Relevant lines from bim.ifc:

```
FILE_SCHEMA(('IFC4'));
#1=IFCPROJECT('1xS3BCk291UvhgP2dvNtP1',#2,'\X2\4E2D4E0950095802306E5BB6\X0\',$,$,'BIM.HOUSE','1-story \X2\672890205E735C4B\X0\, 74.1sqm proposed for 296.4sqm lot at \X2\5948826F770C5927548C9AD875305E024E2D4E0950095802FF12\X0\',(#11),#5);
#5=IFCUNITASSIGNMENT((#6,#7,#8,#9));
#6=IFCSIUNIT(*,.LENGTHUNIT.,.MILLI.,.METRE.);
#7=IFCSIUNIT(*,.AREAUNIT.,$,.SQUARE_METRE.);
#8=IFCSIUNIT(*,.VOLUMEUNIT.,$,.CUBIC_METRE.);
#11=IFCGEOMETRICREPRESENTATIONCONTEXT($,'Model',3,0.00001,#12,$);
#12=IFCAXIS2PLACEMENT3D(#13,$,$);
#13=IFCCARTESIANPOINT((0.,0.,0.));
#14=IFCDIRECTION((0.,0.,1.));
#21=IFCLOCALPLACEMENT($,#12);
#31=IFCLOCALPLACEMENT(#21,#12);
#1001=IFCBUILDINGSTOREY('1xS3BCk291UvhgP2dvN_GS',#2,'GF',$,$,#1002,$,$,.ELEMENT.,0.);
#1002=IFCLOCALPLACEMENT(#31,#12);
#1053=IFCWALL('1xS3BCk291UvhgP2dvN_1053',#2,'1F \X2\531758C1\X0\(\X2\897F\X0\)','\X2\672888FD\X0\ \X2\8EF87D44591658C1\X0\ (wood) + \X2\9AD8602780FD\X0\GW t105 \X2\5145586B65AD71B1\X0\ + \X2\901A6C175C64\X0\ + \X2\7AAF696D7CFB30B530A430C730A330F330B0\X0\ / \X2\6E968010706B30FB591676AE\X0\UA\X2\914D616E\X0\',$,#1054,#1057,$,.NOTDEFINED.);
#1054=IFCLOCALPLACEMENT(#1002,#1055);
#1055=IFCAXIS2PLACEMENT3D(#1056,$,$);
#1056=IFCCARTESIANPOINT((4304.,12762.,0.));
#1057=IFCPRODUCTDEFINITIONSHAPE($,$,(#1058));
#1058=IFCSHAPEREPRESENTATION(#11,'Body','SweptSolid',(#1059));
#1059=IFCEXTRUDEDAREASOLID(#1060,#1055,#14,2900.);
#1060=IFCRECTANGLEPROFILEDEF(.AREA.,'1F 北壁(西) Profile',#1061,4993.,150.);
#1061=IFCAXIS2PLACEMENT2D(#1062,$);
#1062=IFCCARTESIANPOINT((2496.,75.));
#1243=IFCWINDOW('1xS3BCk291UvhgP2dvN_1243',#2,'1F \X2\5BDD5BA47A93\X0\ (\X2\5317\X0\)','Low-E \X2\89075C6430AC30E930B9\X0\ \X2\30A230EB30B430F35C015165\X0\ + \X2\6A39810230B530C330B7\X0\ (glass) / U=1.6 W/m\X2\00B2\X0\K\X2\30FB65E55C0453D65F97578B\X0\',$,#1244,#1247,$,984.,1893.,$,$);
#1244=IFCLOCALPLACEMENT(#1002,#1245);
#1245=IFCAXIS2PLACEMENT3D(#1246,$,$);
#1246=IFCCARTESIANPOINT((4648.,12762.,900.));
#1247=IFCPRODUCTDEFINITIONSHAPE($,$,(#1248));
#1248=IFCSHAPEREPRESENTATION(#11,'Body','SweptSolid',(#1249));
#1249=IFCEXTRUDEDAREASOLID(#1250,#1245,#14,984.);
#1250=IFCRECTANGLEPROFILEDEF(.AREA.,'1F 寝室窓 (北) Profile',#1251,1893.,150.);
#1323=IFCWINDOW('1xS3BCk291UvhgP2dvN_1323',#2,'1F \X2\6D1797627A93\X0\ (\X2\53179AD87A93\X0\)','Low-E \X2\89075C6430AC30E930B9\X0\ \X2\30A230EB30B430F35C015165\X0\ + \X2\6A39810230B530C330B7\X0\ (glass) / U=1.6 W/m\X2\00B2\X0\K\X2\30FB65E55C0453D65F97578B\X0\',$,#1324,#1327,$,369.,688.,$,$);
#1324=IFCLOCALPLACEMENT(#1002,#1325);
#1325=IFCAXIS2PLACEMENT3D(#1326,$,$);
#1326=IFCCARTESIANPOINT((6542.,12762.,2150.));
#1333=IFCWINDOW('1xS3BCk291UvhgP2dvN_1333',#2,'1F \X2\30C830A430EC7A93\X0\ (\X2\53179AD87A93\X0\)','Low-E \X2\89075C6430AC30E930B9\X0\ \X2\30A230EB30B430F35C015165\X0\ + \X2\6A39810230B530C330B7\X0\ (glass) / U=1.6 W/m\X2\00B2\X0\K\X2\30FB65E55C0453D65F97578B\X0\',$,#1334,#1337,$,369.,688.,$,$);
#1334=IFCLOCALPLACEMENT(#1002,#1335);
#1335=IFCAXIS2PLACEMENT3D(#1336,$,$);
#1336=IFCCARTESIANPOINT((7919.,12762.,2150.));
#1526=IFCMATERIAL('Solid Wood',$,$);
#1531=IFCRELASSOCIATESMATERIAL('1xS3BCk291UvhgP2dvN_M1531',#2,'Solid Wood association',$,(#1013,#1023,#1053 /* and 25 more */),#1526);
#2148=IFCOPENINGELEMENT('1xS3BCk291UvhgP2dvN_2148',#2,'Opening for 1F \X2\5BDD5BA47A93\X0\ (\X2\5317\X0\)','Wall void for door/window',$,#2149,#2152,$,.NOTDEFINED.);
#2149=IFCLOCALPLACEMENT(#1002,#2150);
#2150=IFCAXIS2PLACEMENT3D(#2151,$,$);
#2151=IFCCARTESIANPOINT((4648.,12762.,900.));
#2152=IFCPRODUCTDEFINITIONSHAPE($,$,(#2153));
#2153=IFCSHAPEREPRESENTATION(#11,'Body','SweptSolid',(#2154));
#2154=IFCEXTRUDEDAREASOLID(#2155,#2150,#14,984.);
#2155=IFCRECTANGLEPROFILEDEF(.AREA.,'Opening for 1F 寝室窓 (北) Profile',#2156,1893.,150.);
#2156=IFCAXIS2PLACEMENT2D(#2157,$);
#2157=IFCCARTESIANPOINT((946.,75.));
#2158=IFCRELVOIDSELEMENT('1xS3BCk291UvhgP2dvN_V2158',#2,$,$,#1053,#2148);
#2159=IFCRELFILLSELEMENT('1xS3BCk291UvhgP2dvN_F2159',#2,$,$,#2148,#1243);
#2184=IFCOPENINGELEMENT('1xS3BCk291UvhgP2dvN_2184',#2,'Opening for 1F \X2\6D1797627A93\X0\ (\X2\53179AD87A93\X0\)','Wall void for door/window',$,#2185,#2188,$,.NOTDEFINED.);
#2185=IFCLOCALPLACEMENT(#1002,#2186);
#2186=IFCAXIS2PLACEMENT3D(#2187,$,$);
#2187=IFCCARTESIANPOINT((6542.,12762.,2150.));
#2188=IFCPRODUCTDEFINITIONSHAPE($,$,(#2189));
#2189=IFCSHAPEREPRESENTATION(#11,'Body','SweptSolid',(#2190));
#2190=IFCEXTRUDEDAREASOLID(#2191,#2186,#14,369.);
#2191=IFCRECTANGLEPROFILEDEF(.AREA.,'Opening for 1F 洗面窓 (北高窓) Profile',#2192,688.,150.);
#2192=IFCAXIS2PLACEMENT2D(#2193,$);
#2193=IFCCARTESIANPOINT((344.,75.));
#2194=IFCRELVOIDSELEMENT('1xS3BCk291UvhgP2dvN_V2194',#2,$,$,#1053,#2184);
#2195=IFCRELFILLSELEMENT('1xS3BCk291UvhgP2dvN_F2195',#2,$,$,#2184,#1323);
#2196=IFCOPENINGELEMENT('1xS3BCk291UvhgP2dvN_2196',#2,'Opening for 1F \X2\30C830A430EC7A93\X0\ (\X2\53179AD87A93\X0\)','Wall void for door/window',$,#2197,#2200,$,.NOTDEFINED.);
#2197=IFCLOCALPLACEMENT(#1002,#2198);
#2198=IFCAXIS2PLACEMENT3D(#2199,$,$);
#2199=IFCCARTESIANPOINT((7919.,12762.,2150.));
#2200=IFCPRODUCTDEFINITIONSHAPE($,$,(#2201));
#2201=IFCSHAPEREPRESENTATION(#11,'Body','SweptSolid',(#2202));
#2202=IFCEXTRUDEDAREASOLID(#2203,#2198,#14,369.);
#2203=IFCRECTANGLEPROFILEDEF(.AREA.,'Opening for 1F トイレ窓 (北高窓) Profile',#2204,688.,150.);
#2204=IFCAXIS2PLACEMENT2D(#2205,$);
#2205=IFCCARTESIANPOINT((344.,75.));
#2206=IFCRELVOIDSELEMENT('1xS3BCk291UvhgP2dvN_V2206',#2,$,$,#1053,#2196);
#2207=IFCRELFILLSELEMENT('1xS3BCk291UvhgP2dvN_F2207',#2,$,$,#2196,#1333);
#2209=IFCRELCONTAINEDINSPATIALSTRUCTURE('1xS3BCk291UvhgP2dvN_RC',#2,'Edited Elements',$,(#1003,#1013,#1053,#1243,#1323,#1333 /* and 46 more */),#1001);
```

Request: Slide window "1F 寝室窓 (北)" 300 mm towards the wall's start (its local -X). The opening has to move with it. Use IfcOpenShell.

```python
import ifcopenshell
import ifcopenshell.api.geometry
import ifcopenshell.util.placement

model = ifcopenshell.open("bim.ifc")

window = model.by_id(1243)
opening = window.FillsVoids[0].RelatingOpeningElement
wall = opening.VoidsElements[0].RelatingBuildingElement

wall_matrix = ifcopenshell.util.placement.get_local_placement(wall.ObjectPlacement)
shift = wall_matrix[:3, 0] * -300.0
before = ifcopenshell.util.placement.get_local_placement(window.ObjectPlacement)[:3, 3].copy()

# The window is not placed relative to its opening, so move both.
for product in (opening, window):
    matrix = ifcopenshell.util.placement.get_local_placement(product.ObjectPlacement)
    matrix[:3, 3] += shift
    ifcopenshell.api.geometry.edit_object_placement(model, product=product, matrix=matrix, is_si=False)

after = ifcopenshell.util.placement.get_local_placement(window.ObjectPlacement)[:3, 3]
print("window moved by", (after - before).round(3) + 0.0)

model.write("bim-out.ifc")
```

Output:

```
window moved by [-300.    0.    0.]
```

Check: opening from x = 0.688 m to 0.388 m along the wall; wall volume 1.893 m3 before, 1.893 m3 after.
